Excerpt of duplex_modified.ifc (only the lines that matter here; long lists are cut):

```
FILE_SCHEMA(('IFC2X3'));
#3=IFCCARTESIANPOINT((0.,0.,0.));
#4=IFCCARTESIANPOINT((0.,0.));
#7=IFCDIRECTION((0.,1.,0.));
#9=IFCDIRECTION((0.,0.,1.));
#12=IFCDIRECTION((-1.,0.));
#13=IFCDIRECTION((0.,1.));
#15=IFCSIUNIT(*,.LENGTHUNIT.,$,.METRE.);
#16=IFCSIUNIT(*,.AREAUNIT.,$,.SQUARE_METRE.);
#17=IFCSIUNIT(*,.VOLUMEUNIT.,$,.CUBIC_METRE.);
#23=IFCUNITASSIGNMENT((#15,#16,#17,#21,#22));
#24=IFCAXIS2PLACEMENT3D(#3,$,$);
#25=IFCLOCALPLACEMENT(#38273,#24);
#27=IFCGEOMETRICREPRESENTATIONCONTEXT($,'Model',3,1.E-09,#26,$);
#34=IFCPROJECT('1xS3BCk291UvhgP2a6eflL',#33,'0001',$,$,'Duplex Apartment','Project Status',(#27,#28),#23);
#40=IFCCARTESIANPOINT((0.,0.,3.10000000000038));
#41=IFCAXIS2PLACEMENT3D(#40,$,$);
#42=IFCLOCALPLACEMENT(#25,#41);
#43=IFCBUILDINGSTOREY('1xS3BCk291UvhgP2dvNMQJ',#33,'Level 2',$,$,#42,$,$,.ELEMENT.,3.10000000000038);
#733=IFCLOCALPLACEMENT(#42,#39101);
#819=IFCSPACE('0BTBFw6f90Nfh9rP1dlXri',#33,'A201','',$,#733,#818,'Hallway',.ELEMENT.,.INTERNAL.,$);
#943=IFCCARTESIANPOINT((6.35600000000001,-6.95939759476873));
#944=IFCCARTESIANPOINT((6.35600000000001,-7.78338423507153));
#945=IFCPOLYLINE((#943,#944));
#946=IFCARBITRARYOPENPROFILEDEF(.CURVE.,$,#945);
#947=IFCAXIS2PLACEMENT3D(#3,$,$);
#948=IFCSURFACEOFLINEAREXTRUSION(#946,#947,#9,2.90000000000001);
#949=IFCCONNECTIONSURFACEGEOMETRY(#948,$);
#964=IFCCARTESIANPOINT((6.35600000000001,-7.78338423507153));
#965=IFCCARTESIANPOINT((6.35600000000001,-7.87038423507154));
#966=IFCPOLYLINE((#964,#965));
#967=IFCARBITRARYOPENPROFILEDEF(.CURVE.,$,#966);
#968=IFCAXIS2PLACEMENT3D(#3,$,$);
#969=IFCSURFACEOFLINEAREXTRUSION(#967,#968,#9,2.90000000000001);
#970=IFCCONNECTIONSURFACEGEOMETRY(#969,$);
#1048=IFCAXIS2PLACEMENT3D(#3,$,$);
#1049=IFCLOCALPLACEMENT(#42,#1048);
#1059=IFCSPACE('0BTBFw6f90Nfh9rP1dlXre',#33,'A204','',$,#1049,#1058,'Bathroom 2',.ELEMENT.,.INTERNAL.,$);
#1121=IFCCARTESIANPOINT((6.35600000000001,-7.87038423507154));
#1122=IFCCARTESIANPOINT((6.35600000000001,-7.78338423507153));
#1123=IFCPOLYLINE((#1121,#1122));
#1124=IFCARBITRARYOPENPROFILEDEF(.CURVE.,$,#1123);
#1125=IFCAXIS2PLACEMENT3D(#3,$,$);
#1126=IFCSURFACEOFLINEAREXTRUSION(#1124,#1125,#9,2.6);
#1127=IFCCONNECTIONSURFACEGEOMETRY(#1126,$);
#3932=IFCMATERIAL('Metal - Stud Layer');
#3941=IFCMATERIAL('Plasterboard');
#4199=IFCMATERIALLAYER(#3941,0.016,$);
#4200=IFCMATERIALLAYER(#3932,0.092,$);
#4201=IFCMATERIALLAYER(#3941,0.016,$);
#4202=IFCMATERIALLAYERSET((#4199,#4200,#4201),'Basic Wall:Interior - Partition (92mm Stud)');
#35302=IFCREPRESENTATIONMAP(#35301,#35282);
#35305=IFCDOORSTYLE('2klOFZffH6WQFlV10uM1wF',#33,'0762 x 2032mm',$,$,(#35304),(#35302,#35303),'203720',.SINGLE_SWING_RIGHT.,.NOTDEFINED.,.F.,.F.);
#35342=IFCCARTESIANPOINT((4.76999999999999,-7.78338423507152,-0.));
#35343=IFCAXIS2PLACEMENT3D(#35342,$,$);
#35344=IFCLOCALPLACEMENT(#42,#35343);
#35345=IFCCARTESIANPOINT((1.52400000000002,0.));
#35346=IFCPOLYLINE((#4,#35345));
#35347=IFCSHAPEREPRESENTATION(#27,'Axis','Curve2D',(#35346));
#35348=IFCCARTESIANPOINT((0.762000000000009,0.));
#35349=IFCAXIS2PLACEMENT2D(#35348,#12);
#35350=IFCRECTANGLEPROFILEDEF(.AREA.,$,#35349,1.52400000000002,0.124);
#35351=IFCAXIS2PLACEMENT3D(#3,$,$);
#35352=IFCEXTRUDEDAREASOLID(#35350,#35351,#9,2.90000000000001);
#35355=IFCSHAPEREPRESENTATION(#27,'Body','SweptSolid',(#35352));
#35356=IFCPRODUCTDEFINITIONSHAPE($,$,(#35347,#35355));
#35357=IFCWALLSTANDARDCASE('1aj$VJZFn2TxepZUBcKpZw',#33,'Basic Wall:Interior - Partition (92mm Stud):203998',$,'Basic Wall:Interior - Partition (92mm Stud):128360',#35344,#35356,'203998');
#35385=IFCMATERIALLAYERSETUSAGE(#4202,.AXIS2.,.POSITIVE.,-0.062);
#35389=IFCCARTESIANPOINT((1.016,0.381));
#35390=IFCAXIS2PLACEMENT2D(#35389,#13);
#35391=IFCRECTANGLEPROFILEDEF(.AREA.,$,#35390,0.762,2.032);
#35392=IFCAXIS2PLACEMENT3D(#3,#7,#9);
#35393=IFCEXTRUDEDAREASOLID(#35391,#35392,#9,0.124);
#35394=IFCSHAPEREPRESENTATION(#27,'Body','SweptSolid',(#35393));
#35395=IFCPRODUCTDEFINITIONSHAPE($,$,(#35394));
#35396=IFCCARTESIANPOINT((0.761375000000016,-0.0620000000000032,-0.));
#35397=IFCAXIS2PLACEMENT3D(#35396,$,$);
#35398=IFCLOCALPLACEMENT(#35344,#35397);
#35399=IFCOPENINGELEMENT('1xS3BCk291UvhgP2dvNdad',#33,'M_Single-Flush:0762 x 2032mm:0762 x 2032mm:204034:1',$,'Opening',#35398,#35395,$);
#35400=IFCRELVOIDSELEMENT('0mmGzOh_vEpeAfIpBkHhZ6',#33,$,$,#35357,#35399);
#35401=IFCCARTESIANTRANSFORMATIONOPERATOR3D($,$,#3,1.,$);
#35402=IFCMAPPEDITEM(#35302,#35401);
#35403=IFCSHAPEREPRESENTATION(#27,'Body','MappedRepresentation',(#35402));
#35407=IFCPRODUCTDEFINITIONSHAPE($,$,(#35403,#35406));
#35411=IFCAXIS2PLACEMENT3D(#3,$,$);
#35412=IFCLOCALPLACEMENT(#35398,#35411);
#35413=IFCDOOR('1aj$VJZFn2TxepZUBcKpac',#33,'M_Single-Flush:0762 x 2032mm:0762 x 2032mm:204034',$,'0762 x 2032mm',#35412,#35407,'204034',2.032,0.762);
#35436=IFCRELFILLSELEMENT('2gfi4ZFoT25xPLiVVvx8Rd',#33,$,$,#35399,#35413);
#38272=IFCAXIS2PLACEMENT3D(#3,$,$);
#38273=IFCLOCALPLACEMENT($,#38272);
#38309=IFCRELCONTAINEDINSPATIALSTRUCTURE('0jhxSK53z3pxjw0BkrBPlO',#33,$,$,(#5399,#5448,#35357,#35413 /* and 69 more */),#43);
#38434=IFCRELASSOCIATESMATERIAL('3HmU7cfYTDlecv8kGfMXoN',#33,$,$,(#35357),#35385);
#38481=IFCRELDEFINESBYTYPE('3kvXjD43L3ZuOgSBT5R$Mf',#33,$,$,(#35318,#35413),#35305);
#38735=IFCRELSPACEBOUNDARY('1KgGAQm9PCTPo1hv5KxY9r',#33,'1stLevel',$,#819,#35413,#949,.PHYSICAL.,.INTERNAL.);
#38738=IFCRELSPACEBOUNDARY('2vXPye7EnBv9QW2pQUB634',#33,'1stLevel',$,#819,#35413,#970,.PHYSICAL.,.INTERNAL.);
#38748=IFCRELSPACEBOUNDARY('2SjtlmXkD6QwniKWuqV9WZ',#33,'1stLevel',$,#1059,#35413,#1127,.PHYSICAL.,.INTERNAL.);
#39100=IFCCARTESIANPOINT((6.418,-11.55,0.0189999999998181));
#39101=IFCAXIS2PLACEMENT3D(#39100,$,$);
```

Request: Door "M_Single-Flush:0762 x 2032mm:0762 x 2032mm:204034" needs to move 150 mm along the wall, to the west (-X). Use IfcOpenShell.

```python
import numpy as np
import ifcopenshell
import ifcopenshell.api.geometry
import ifcopenshell.util.placement
import ifcopenshell.util.unit

model = ifcopenshell.open("duplex_modified.ifc")
unit_scale = ifcopenshell.util.unit.calculate_unit_scale(model)

door = model.by_guid("1aj$VJZFn2TxepZUBcKpac")
opening = door.FillsVoids[0].RelatingOpeningElement
wall = opening.VoidsElements[0].RelatingBuildingElement

wall_matrix = ifcopenshell.util.placement.get_local_placement(wall.ObjectPlacement)
shift = wall_matrix[:3, 0] * -0.15 / unit_scale
before = ifcopenshell.util.placement.get_local_placement(door.ObjectPlacement)[:3, 3].copy()

# The door is placed relative to its opening, so it follows when the opening moves.
matrix = ifcopenshell.util.placement.get_local_placement(opening.ObjectPlacement)
matrix[:3, 3] += shift
ifcopenshell.api.geometry.edit_object_placement(
    model, product=opening, matrix=matrix, is_si=False, should_transform_children=True
)

# Space boundary surfaces are stored in each space's coordinates; move them too.
for rel in door.ProvidesBoundaries:
    if not rel.ConnectionGeometry:
        continue
    surface = rel.ConnectionGeometry.SurfaceOnRelatingElement
    space_matrix = ifcopenshell.util.placement.get_local_placement(rel.RelatingSpace.ObjectPlacement)
    point = np.array(surface.Position.Location.Coordinates) + space_matrix[:3, :3].T @ shift
    surface.Position = model.createIfcAxis2Placement3D(
        model.createIfcCartesianPoint(point.tolist()), surface.Position.Axis, surface.Position.RefDirection
    )

after = ifcopenshell.util.placement.get_local_placement(door.ObjectPlacement)[:3, 3]
print("door moved by", (after - before).round(3) + 0.0)

model.write("duplex_modified_updated.ifc")
```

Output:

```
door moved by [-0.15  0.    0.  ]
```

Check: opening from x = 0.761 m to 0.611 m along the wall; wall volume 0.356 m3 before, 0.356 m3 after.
